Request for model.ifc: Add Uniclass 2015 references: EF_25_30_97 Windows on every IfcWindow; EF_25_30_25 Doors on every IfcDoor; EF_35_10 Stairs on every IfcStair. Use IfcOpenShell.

First a look at what the model holds.

```python
import ifcopenshell

model = ifcopenshell.open("model.ifc")
print(model.schema)
print("classifications:", [c.Name for c in model.by_type("IfcClassification")])
for ifc_class in ("IfcDoor", "IfcRoof", "IfcStair", "IfcWall", "IfcWindow"):
    print(ifc_class, len(model.by_type(ifc_class)))
```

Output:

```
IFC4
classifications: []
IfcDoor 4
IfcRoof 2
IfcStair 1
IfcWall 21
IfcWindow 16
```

```python
import ifcopenshell
import ifcopenshell.api.classification

model = ifcopenshell.open("model.ifc")

system = ifcopenshell.api.classification.add_classification(model, classification="Uniclass 2015")

codes = {
    "IfcWindow": ("EF_25_30_97", "Windows"),
    "IfcDoor": ("EF_25_30_25", "Doors"),
    "IfcStair": ("EF_35_10", "Stairs"),
}
for ifc_class, (code, name) in codes.items():
    products = model.by_type(ifc_class)
    ifcopenshell.api.classification.add_reference(
        model, products=products, classification=system, identification=code, name=name
    )
    print(code, len(products))

model.write("model_rev.ifc")
```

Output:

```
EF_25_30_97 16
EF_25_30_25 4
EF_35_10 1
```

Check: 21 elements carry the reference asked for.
